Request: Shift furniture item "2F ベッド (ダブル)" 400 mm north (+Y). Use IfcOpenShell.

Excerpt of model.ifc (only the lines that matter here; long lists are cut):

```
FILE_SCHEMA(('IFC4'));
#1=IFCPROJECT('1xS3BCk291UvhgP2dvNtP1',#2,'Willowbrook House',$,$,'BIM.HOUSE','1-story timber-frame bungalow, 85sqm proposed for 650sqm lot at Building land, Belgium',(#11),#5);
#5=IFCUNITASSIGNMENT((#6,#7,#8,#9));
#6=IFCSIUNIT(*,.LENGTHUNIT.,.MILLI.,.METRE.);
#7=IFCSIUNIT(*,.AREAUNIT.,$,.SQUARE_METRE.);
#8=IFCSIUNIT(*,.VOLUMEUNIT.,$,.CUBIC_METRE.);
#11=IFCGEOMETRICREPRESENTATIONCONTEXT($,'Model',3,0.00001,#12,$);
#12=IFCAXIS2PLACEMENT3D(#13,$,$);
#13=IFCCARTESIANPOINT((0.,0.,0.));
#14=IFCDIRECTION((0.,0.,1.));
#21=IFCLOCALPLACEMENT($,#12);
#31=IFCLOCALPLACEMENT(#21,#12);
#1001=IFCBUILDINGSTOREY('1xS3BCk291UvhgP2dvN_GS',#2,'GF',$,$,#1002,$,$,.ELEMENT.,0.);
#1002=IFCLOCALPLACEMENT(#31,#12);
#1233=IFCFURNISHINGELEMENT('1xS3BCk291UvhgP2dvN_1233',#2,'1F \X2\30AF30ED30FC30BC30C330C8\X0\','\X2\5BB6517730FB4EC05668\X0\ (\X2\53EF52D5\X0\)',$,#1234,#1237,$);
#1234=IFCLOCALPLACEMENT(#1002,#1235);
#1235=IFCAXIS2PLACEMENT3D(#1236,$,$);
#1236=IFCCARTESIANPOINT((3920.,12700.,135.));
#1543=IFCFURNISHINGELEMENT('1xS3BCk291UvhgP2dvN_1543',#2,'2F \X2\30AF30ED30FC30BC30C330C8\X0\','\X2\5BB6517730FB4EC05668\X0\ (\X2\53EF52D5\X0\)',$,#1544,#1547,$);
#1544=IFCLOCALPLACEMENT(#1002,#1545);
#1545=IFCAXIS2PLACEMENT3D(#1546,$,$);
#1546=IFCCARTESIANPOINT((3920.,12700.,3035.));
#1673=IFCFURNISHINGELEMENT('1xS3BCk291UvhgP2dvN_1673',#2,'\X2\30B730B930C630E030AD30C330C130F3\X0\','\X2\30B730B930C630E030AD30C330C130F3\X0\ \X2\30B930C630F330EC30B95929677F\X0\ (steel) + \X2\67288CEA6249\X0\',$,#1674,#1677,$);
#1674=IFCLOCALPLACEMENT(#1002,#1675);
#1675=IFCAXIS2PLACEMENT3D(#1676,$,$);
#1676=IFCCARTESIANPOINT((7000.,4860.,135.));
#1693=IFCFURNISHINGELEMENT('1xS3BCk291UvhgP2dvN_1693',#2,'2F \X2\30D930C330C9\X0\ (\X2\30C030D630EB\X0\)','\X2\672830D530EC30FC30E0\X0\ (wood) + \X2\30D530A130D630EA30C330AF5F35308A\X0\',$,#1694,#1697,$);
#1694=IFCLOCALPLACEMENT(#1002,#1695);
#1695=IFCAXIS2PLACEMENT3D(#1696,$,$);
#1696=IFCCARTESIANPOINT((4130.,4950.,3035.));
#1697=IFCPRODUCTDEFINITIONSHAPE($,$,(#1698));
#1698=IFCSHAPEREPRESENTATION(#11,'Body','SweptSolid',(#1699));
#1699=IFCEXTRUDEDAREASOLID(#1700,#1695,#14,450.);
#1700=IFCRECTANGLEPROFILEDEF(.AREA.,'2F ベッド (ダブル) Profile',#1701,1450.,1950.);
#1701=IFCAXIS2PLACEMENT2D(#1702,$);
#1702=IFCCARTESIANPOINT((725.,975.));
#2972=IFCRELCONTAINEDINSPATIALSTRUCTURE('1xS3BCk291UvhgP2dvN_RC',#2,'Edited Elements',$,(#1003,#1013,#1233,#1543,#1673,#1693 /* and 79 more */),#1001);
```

```python
import ifcopenshell
import ifcopenshell.api.geometry
import ifcopenshell.util.placement

model = ifcopenshell.open("model.ifc")

item = model.by_guid("1xS3BCk291UvhgP2dvN_1693")
matrix = ifcopenshell.util.placement.get_local_placement(item.ObjectPlacement)
matrix[1, 3] += 400.0
ifcopenshell.api.geometry.edit_object_placement(model, product=item, matrix=matrix, is_si=False)

print(ifcopenshell.util.placement.get_local_placement(item.ObjectPlacement).round(3) + 0.0)

model.write("model_updated.ifc")
```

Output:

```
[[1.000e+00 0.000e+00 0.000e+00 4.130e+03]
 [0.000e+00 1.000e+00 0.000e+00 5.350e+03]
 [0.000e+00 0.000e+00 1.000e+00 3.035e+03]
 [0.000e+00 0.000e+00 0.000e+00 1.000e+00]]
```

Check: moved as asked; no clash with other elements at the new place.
